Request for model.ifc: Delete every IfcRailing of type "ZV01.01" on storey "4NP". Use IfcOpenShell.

First a look at what the model holds.

```python
import ifcopenshell
import ifcopenshell.util.element

model = ifcopenshell.open("model.ifc")
print(model.schema)
storey = next(s for s in model.by_type("IfcBuildingStorey") if s.Name == "4NP")
railings = [e for e in ifcopenshell.util.element.get_decomposition(storey) if e.is_a("IfcRailing")]
seen = {}
for e in railings:
    element_type = ifcopenshell.util.element.get_type(e)
    name = element_type.Name if element_type not in (None, e) else None
    seen[name] = seen.get(name, 0) + 1
for name, count in sorted(seen.items(), key=str):
    print(count, "x", name)
```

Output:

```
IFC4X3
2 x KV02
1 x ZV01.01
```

```python
import ifcopenshell
import ifcopenshell.api.root
import ifcopenshell.util.element

model = ifcopenshell.open("model.ifc")

storey = next(s for s in model.by_type("IfcBuildingStorey") if s.Name == "4NP")
railings = [e for e in ifcopenshell.util.element.get_decomposition(storey) if e.is_a("IfcRailing")]
targets = [e for e in railings if (t := ifcopenshell.util.element.get_type(e)) not in (None, e) and t.Name == "ZV01.01"]

for e in targets:
    ifcopenshell.api.root.remove_product(model, product=e)
print(len(targets), "removed")

model.write("model_v2.ifc")
```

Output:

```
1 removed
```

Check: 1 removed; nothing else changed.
